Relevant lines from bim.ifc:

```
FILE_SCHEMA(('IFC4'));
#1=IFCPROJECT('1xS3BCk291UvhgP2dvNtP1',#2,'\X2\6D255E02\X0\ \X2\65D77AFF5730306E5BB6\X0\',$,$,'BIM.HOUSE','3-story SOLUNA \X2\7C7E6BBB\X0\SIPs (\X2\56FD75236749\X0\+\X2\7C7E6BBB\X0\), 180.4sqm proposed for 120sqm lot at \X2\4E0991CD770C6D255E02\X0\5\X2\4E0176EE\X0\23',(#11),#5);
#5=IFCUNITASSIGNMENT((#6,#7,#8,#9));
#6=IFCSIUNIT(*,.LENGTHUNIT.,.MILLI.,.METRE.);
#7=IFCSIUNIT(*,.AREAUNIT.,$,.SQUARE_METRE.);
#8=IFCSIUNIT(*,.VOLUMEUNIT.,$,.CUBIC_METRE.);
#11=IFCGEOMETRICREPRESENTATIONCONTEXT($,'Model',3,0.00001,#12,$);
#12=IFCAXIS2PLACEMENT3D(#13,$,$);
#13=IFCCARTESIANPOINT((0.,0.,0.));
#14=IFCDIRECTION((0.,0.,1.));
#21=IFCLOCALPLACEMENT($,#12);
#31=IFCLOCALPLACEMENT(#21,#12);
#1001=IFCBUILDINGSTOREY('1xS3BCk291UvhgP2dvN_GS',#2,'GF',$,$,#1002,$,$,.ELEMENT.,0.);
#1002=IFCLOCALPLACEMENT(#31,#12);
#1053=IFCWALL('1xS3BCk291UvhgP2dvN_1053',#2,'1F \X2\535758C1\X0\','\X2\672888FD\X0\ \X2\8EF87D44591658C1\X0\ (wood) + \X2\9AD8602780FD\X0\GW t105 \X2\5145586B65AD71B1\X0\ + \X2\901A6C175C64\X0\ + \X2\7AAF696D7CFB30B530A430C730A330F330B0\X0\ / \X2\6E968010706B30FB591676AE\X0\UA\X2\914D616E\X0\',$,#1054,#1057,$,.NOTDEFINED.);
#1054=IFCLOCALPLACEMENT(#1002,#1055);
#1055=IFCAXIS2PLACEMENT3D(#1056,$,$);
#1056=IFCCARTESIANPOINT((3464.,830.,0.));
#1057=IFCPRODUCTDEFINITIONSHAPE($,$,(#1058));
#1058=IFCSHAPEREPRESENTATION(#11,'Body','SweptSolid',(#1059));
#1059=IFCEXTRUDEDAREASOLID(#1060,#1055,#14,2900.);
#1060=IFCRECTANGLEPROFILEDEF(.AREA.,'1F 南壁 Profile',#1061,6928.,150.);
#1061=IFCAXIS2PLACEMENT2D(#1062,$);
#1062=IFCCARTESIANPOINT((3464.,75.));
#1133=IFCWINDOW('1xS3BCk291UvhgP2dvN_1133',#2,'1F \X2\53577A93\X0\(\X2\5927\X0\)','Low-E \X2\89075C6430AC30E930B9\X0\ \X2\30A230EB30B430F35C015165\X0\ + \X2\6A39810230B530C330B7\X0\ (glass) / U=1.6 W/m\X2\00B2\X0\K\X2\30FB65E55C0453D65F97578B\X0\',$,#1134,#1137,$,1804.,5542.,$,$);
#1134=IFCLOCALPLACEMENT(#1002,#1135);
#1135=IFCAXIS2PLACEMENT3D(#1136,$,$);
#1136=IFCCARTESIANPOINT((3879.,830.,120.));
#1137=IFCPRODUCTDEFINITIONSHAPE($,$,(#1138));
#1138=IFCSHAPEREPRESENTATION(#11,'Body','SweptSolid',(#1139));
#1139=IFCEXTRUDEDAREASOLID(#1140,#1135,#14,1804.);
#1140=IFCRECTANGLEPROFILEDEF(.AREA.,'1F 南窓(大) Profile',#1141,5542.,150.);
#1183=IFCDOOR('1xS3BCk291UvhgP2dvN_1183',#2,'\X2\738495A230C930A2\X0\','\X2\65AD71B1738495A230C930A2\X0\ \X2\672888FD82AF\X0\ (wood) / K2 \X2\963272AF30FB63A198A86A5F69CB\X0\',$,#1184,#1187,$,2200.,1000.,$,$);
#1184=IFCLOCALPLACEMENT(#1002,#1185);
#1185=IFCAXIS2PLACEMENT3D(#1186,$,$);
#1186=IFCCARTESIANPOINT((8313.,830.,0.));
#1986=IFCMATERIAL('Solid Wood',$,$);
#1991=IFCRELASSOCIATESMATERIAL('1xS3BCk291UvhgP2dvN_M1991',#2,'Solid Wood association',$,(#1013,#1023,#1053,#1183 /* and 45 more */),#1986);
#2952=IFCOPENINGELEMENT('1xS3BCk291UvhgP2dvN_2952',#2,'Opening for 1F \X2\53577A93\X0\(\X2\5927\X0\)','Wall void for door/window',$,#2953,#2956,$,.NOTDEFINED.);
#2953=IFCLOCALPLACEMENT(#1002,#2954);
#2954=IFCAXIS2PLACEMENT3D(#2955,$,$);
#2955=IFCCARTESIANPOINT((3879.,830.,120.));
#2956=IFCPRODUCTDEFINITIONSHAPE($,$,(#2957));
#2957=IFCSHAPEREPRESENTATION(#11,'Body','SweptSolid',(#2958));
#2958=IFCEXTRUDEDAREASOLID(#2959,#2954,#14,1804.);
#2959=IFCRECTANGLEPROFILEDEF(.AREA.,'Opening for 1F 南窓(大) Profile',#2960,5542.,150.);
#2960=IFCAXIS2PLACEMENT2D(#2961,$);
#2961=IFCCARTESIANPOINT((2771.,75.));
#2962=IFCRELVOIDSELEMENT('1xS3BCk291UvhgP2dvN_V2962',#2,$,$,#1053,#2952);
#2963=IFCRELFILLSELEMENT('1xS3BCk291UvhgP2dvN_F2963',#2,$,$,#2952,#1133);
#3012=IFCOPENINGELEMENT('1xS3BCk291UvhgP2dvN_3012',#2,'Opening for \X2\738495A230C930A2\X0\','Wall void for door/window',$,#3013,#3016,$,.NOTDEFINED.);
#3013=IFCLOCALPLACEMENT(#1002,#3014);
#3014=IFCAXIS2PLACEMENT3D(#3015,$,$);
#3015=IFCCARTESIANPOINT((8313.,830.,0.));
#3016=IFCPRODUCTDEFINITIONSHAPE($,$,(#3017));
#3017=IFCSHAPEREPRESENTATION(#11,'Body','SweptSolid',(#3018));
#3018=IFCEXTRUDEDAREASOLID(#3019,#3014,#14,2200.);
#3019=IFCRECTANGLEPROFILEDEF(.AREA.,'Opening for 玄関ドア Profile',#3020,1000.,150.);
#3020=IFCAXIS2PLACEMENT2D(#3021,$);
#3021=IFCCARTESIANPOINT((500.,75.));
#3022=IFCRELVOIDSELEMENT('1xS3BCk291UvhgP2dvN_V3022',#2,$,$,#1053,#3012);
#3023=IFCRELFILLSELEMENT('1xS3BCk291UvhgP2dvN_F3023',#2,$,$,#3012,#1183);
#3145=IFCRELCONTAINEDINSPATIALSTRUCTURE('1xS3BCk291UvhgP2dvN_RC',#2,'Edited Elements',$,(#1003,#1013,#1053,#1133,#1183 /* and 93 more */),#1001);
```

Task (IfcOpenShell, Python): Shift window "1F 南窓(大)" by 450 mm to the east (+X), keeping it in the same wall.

```python
import ifcopenshell
import ifcopenshell.api.geometry
import ifcopenshell.util.placement

model = ifcopenshell.open("bim.ifc")

window = model.by_guid("1xS3BCk291UvhgP2dvN_1133")
opening = window.FillsVoids[0].RelatingOpeningElement
wall = opening.VoidsElements[0].RelatingBuildingElement

wall_matrix = ifcopenshell.util.placement.get_local_placement(wall.ObjectPlacement)
shift = wall_matrix[:3, 0] * 450.0
before = ifcopenshell.util.placement.get_local_placement(window.ObjectPlacement)[:3, 3].copy()

# The window is not placed relative to its opening, so move both.
for product in (opening, window):
    matrix = ifcopenshell.util.placement.get_local_placement(product.ObjectPlacement)
    matrix[:3, 3] += shift
    ifcopenshell.api.geometry.edit_object_placement(model, product=product, matrix=matrix, is_si=False)

after = ifcopenshell.util.placement.get_local_placement(window.ObjectPlacement)[:3, 3]
print("window moved by", (after - before).round(3) + 0.0)

model.write("bim_updated.ifc")
```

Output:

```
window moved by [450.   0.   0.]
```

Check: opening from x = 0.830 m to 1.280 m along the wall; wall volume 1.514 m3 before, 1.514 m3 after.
